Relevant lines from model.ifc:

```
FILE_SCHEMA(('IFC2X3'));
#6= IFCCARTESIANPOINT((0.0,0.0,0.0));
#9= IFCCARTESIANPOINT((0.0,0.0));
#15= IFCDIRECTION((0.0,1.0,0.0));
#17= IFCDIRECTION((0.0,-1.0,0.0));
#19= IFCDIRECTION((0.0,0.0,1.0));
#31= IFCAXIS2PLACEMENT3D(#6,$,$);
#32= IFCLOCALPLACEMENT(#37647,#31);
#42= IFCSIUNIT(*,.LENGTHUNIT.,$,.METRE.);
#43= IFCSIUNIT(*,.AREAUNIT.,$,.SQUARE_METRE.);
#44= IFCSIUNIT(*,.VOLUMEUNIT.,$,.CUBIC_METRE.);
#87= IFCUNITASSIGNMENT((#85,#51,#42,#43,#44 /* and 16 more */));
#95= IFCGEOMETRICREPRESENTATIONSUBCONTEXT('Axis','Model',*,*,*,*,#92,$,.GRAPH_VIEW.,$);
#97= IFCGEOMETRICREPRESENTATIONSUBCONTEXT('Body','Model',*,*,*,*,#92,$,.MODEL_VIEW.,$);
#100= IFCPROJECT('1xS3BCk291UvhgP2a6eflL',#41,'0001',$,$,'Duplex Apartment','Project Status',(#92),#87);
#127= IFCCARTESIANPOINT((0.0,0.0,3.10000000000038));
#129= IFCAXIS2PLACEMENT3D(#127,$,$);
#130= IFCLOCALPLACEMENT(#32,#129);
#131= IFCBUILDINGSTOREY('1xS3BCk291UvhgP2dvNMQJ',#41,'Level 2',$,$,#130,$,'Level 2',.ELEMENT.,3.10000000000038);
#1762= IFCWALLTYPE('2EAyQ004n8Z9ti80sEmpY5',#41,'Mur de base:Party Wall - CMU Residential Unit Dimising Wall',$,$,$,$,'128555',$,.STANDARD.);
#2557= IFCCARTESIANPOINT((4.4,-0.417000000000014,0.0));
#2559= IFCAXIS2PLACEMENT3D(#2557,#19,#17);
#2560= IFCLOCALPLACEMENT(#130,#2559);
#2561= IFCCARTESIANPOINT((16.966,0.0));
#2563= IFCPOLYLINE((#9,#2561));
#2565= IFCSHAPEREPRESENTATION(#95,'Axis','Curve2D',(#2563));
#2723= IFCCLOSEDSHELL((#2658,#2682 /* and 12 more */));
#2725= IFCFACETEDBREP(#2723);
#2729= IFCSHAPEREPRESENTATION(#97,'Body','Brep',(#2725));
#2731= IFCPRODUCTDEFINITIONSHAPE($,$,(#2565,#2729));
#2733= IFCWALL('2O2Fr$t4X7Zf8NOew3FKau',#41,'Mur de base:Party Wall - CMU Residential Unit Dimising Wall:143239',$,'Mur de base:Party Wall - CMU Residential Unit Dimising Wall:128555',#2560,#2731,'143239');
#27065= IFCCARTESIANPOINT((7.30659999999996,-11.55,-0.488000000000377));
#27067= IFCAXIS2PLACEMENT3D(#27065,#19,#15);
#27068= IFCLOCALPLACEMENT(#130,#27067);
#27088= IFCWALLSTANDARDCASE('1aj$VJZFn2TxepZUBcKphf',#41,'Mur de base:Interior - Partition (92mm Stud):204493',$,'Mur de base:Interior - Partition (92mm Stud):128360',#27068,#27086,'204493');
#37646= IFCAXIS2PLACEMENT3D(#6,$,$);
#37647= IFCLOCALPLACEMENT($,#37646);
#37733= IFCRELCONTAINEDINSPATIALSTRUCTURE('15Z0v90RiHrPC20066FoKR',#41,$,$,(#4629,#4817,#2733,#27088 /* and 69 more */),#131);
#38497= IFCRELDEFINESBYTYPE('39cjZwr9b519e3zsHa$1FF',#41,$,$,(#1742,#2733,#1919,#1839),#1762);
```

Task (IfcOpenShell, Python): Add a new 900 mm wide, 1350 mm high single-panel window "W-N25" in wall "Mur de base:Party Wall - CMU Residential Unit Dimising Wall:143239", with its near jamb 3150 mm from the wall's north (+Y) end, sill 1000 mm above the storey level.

```python
import numpy as np
import ifcopenshell
import ifcopenshell.api.feature
import ifcopenshell.api.geometry
import ifcopenshell.api.root
import ifcopenshell.api.spatial
import ifcopenshell.api.type
import ifcopenshell.geom
import ifcopenshell.util.element
import ifcopenshell.util.placement
import ifcopenshell.util.representation
import ifcopenshell.util.shape
import ifcopenshell.util.unit

model = ifcopenshell.open("model.ifc")
unit_scale = ifcopenshell.util.unit.calculate_unit_scale(model)
settings = ifcopenshell.geom.settings()


def volume(element):
    """Net volume in cubic metres, openings subtracted."""
    shape = ifcopenshell.geom.create_shape(settings, element)
    return ifcopenshell.util.shape.get_volume(shape.geometry)


wall = model.by_guid("2O2Fr$t4X7Zf8NOew3FKau")
storey = ifcopenshell.util.element.get_container(wall, ifc_class="IfcBuildingStorey")
context = ifcopenshell.util.representation.get_context(model, "Model", "Body", "MODEL_VIEW")
before = volume(wall)

width, height, from_end, sill = 0.9, 1.35, 3.15, 1  # metres

# The wall runs along its own X axis, and the end named is its -X end.
wall_shape = ifcopenshell.geom.create_shape(settings, wall)
x, y, z = ifcopenshell.util.shape.get_vertices(wall_shape.geometry).T
start = x.min() + from_end
face, thickness = float(y.min()), float(y.max() - y.min())
wall_matrix = ifcopenshell.util.placement.get_local_placement(wall.ObjectPlacement)
level = ifcopenshell.util.placement.get_local_placement(storey.ObjectPlacement)[2, 3]


def in_wall(x, y):
    """Placement at x, y metres in the wall's axes, at sill height."""
    matrix = wall_matrix.copy()
    matrix[:, 3] = wall_matrix @ np.array([x / unit_scale, y / unit_scale, 0.0, 1.0])
    matrix[2, 3] = level + sill / unit_scale
    return matrix


# Opening: a box that overshoots both wall faces by 50 mm.
opening = ifcopenshell.api.root.create_entity(model, ifc_class="IfcOpeningElement")
box = ifcopenshell.api.geometry.add_wall_representation(
    model, context=context, length=width, height=height, thickness=thickness + 0.1
)
ifcopenshell.api.geometry.assign_representation(model, product=opening, representation=box)
ifcopenshell.api.geometry.edit_object_placement(model, product=opening, matrix=in_wall(start, face - 0.05), is_si=False)
ifcopenshell.api.feature.add_feature(model, feature=opening, element=wall)

window = ifcopenshell.api.root.create_entity(model, ifc_class="IfcWindow", name="W-N25")
window.OverallWidth, window.OverallHeight = width / unit_scale, height / unit_scale
body = ifcopenshell.api.geometry.add_window_representation(
    model,
    context=context,
    overall_width=window.OverallWidth,
    overall_height=window.OverallHeight,
    partition_type="SINGLE_PANEL",
)
ifcopenshell.api.geometry.assign_representation(model, product=window, representation=body)
ifcopenshell.api.spatial.assign_container(model, products=[window], relating_structure=storey)
fills = ifcopenshell.api.feature.add_filling(model, opening=opening, element=window)
fills.OwnerHistory = window.OwnerHistory  # required in IFC2X3

# IFC2X3 keeps the operation on the window style.
style = ifcopenshell.api.root.create_entity(model, ifc_class="IfcWindowStyle", name="W-N25")
style.OperationType, style.ConstructionType = "SINGLE_PANEL", "NOTDEFINED"
style.ParameterTakesPrecedence = style.Sizeable = False
ifcopenshell.api.type.assign_type(model, related_objects=[window], relating_type=style)

# Centre the window in the wall's thickness.
ifcopenshell.api.geometry.edit_object_placement(model, product=window, matrix=in_wall(start, face), is_si=False)
window_shape = ifcopenshell.geom.create_shape(settings, window)
depth = ifcopenshell.util.shape.get_vertices(window_shape.geometry)[:, 1]
offset = face + thickness / 2 - (depth.min() + depth.max()) / 2
ifcopenshell.api.geometry.edit_object_placement(model, product=window, matrix=in_wall(start, offset), is_si=False)

after = volume(wall)

print(f"wall volume {before:.3f} -> {after:.3f} m3")

model.write("model_updated.ifc")
```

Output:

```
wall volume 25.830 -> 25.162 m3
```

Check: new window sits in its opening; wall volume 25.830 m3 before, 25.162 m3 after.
